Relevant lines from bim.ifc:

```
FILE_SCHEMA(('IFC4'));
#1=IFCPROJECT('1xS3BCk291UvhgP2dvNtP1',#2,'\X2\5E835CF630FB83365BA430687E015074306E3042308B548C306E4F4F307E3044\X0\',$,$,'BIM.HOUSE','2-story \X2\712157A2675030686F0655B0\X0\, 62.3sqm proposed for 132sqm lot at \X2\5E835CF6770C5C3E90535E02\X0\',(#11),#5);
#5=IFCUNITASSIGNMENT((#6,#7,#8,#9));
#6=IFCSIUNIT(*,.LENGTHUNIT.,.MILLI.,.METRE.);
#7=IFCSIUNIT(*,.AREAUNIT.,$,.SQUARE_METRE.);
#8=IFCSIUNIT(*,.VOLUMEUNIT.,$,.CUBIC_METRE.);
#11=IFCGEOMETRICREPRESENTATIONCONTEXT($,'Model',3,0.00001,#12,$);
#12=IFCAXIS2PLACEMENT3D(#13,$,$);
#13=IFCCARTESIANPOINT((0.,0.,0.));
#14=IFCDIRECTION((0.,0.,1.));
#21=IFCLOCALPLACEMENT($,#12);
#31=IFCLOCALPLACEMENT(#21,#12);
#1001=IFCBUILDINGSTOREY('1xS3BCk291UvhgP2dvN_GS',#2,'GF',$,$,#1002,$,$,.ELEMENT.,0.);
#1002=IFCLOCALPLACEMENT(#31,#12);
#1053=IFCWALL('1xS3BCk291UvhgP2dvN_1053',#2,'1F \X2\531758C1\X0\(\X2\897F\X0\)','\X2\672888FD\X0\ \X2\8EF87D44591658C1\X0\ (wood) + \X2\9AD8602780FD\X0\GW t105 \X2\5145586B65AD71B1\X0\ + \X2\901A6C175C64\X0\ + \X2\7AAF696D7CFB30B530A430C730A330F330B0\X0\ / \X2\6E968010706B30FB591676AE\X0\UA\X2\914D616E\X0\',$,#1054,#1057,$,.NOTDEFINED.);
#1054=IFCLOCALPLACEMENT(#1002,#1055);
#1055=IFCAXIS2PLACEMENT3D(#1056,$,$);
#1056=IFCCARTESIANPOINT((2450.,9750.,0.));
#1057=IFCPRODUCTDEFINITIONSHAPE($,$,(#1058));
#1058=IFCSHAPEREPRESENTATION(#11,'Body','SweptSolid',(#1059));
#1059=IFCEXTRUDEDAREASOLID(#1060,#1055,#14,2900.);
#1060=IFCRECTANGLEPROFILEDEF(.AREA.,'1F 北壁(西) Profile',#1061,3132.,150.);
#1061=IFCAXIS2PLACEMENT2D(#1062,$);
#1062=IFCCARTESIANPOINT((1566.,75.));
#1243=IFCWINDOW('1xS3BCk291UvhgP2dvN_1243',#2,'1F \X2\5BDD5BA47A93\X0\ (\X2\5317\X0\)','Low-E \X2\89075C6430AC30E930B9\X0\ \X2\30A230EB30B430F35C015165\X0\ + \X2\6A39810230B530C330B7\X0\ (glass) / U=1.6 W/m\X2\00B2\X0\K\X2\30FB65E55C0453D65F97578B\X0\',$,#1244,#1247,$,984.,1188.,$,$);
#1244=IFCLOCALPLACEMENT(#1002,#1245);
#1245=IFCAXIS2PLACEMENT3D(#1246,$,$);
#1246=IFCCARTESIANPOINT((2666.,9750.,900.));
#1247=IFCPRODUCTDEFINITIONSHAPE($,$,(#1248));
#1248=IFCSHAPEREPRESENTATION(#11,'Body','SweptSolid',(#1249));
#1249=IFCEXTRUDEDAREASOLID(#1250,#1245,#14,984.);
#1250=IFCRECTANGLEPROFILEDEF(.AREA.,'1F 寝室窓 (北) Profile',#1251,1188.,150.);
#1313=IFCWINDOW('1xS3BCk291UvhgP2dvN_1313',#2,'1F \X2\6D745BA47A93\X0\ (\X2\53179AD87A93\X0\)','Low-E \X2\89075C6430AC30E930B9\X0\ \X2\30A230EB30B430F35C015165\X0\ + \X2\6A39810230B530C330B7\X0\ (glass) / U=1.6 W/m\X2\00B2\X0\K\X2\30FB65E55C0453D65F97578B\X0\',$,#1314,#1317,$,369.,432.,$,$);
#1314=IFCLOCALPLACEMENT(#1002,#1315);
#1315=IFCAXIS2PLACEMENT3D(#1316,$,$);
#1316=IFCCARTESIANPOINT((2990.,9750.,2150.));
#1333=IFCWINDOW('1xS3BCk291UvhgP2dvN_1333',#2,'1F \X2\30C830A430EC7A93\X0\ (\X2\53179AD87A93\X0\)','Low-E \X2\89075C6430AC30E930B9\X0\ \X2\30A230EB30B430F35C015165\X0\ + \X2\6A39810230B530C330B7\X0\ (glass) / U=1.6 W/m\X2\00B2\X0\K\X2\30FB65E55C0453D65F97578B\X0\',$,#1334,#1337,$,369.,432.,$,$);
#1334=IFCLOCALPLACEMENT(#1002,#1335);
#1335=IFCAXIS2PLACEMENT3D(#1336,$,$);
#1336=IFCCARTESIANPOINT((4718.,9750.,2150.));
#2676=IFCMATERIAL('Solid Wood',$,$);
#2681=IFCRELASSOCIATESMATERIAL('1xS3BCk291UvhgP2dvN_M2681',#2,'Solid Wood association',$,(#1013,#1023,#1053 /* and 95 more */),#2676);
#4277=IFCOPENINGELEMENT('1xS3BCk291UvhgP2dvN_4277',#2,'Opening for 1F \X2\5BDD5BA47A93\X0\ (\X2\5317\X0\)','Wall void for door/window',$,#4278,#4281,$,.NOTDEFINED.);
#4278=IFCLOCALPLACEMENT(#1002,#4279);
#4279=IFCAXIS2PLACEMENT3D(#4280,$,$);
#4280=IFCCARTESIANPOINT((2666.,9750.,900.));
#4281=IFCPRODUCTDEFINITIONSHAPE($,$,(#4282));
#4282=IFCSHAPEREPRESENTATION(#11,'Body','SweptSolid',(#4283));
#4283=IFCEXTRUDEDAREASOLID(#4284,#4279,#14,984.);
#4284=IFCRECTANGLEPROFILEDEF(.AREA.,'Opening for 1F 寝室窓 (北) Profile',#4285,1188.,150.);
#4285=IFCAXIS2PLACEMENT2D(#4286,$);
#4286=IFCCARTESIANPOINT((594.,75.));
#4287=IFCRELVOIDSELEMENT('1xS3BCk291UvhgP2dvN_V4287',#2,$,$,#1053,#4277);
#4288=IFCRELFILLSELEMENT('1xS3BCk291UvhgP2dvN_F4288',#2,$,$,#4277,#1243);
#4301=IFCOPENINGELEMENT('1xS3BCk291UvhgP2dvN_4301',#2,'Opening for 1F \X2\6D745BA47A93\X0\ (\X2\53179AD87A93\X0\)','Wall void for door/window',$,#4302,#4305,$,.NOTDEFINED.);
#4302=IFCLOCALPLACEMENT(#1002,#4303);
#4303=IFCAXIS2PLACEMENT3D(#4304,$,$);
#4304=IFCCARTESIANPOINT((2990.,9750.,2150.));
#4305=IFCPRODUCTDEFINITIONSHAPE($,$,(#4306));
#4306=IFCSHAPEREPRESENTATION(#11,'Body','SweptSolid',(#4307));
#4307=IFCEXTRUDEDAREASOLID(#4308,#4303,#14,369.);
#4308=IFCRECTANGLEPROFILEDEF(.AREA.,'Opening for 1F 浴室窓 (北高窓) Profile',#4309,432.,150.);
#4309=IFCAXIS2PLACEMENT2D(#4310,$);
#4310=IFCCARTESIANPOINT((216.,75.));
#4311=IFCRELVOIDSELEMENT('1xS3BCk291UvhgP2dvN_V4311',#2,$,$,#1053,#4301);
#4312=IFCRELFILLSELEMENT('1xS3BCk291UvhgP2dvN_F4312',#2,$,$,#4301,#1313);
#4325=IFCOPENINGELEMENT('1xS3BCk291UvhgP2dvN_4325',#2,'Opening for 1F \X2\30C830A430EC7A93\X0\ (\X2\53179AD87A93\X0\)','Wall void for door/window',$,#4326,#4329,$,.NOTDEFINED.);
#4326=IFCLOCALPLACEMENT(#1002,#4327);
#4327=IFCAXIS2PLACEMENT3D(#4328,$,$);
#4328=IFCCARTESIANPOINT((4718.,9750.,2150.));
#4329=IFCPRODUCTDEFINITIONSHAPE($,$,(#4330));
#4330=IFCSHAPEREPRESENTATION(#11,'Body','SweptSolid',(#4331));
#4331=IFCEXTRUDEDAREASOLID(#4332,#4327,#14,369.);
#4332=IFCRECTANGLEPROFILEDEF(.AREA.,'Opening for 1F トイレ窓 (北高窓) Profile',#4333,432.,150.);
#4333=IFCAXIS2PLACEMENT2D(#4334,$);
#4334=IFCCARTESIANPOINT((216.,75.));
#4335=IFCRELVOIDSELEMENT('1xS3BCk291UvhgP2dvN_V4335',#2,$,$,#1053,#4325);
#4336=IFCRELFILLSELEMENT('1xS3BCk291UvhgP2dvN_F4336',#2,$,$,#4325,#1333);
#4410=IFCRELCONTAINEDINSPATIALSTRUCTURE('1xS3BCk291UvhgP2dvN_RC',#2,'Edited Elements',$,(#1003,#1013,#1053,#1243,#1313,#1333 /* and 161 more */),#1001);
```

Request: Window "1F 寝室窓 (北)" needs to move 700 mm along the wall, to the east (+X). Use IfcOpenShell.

```python
import ifcopenshell
import ifcopenshell.api.geometry
import ifcopenshell.util.placement

model = ifcopenshell.open("bim.ifc")

window = model.by_guid("1xS3BCk291UvhgP2dvN_1243")
opening = window.FillsVoids[0].RelatingOpeningElement
wall = opening.VoidsElements[0].RelatingBuildingElement

wall_matrix = ifcopenshell.util.placement.get_local_placement(wall.ObjectPlacement)
shift = wall_matrix[:3, 0] * 700.0
before = ifcopenshell.util.placement.get_local_placement(window.ObjectPlacement)[:3, 3].copy()

# The window is not placed relative to its opening, so move both.
for product in (opening, window):
    matrix = ifcopenshell.util.placement.get_local_placement(product.ObjectPlacement)
    matrix[:3, 3] += shift
    ifcopenshell.api.geometry.edit_object_placement(model, product=product, matrix=matrix, is_si=False)

after = ifcopenshell.util.placement.get_local_placement(window.ObjectPlacement)[:3, 3]
print("window moved by", (after - before).round(3) + 0.0)

model.write("bim_edited.ifc")
```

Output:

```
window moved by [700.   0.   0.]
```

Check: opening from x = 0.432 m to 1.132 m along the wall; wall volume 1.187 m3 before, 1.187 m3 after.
